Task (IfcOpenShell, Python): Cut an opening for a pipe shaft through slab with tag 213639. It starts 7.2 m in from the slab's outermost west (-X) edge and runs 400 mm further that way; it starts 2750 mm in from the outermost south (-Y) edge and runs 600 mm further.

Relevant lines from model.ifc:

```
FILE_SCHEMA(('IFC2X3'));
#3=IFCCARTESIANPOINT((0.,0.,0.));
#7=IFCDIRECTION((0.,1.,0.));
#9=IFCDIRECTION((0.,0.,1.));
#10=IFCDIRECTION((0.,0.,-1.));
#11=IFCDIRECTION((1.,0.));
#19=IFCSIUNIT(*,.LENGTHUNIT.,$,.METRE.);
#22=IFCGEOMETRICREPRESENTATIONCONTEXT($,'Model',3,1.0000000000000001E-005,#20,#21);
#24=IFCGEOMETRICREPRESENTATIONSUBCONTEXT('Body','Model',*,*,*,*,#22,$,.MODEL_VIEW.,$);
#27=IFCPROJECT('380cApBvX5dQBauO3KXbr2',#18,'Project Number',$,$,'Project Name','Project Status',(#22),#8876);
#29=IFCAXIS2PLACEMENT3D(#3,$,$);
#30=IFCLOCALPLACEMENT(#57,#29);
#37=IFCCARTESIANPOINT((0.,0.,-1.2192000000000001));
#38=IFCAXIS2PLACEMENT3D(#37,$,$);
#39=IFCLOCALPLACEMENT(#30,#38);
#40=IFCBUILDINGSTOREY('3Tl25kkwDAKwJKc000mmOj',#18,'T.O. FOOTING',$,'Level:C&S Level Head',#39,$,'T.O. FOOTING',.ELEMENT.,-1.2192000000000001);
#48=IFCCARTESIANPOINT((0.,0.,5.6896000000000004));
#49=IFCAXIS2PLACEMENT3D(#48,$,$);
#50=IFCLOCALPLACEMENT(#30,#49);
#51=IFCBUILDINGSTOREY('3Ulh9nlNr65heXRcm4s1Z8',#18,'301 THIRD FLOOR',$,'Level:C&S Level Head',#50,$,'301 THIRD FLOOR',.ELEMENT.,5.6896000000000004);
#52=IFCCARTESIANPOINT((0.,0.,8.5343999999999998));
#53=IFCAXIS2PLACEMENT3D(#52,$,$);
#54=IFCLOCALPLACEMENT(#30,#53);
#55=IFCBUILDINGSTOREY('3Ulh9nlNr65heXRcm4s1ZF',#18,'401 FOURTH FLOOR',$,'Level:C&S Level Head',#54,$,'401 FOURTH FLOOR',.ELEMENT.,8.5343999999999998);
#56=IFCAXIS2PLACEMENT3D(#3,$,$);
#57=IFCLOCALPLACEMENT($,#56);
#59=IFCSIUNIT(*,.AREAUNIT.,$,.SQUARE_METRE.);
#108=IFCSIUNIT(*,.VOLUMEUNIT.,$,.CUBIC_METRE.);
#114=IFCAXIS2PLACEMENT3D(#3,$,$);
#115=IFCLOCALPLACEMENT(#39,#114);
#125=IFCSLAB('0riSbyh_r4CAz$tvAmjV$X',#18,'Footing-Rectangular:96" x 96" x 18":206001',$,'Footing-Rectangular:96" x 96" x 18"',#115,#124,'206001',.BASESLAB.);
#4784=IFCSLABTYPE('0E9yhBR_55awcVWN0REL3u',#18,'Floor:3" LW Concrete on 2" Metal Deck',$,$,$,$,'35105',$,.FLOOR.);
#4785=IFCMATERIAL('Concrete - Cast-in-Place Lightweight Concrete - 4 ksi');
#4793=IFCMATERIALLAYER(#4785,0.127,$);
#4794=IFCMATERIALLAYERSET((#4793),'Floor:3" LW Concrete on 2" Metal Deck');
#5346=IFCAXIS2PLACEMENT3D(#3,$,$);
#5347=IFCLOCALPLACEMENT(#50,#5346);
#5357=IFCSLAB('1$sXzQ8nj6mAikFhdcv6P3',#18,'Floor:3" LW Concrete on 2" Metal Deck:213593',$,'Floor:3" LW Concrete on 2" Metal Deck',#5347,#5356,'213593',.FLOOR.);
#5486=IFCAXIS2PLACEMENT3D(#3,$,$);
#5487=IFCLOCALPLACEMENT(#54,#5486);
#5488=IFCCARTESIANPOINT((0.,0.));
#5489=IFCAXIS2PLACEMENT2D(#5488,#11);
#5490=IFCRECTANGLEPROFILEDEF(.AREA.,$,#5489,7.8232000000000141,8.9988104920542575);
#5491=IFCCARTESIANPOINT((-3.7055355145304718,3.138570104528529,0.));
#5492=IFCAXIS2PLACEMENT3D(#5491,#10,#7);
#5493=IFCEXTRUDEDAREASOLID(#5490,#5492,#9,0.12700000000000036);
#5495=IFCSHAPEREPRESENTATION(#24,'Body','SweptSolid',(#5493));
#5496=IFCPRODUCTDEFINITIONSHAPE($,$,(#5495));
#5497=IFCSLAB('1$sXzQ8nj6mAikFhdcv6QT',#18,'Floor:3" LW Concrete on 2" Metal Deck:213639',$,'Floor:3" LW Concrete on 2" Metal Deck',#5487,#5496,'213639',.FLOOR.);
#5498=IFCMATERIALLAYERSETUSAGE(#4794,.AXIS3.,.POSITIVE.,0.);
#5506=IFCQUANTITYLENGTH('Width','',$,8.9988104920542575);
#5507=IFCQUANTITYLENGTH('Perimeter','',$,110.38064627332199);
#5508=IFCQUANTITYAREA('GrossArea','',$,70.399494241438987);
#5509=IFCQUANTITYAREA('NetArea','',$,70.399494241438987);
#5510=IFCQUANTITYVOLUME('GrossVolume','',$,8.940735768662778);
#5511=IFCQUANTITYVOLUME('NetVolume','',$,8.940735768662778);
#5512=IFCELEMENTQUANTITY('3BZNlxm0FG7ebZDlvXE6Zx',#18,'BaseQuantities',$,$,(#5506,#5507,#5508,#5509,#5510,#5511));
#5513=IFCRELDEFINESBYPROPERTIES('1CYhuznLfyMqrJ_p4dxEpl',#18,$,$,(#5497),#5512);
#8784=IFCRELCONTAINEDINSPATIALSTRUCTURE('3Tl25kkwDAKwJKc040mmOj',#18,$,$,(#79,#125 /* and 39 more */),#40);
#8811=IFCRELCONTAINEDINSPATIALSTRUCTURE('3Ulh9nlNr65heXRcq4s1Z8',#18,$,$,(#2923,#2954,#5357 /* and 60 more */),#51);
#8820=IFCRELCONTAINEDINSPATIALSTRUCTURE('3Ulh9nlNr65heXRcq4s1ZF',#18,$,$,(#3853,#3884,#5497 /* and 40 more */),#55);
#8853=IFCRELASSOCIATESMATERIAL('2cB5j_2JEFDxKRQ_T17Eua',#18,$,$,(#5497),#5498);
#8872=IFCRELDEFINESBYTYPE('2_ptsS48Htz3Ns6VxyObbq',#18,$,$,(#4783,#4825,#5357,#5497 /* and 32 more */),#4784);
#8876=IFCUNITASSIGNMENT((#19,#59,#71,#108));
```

```python
import numpy as np
import ifcopenshell
import ifcopenshell.api.feature
import ifcopenshell.api.geometry
import ifcopenshell.api.pset
import ifcopenshell.api.root
import ifcopenshell.geom
import ifcopenshell.util.element
import ifcopenshell.util.placement
import ifcopenshell.util.representation
import ifcopenshell.util.shape
import ifcopenshell.util.unit

model = ifcopenshell.open("model.ifc")
unit_scale = ifcopenshell.util.unit.calculate_unit_scale(model)
area_scale = ifcopenshell.util.unit.calculate_unit_scale(model, "AREAUNIT")
volume_scale = ifcopenshell.util.unit.calculate_unit_scale(model, "VOLUMEUNIT")
settings = ifcopenshell.geom.settings()


def volume(element):
    """Net volume in cubic metres, openings subtracted."""
    shape = ifcopenshell.geom.create_shape(settings, element)
    return ifcopenshell.util.shape.get_volume(shape.geometry)


slab = model.by_guid("1$sXzQ8nj6mAikFhdcv6QT")
before = volume(slab)

# Extent in the slab's own axes, in metres. The edges named are its -X and -Y sides.
slab_shape = ifcopenshell.geom.create_shape(settings, slab)
vertices = ifcopenshell.util.shape.get_vertices(slab_shape.geometry)
x_min, y_min, bottom = vertices.min(axis=0)
top = vertices[:, 2].max()

opening = ifcopenshell.api.root.create_entity(model, ifc_class="IfcOpeningElement", name="Pipe shaft opening")
context = ifcopenshell.util.representation.get_context(model, "Model", "Body", "MODEL_VIEW")
width, depth = 0.4, 0.6
outline = [(0.0, 0.0), (width, 0.0), (width, depth), (0.0, depth), (0.0, 0.0)]
# Overshoot both faces by 50 mm so the cut is clean.
shape = ifcopenshell.api.geometry.add_slab_representation(
    model, context=context, depth=top - bottom + 0.1, polyline=outline
)
ifcopenshell.api.geometry.assign_representation(model, product=opening, representation=shape)

matrix = ifcopenshell.util.placement.get_local_placement(slab.ObjectPlacement)
matrix[:, 3] = matrix @ np.append(np.array([x_min + 7.2, y_min + 2.75, bottom - 0.05]) / unit_scale, 1.0)
ifcopenshell.api.geometry.edit_object_placement(model, product=opening, matrix=matrix, is_si=False)
ifcopenshell.api.feature.add_feature(model, feature=opening, element=slab)

after = volume(slab)

# Update the slab's stored quantities.
qto = model.by_id(ifcopenshell.util.element.get_pset(slab, "BaseQuantities", should_inherit=False)["id"])
ifcopenshell.api.pset.edit_qto(model, qto=qto, properties={
    "NetArea": after / (top - bottom) / area_scale,
    "NetVolume": after / volume_scale,
})

print(f"slab volume {before:.3f} -> {after:.3f} m3")

model.write("model_updated.ifc")
```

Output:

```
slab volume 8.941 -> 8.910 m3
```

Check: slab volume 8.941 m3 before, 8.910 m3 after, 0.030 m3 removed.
